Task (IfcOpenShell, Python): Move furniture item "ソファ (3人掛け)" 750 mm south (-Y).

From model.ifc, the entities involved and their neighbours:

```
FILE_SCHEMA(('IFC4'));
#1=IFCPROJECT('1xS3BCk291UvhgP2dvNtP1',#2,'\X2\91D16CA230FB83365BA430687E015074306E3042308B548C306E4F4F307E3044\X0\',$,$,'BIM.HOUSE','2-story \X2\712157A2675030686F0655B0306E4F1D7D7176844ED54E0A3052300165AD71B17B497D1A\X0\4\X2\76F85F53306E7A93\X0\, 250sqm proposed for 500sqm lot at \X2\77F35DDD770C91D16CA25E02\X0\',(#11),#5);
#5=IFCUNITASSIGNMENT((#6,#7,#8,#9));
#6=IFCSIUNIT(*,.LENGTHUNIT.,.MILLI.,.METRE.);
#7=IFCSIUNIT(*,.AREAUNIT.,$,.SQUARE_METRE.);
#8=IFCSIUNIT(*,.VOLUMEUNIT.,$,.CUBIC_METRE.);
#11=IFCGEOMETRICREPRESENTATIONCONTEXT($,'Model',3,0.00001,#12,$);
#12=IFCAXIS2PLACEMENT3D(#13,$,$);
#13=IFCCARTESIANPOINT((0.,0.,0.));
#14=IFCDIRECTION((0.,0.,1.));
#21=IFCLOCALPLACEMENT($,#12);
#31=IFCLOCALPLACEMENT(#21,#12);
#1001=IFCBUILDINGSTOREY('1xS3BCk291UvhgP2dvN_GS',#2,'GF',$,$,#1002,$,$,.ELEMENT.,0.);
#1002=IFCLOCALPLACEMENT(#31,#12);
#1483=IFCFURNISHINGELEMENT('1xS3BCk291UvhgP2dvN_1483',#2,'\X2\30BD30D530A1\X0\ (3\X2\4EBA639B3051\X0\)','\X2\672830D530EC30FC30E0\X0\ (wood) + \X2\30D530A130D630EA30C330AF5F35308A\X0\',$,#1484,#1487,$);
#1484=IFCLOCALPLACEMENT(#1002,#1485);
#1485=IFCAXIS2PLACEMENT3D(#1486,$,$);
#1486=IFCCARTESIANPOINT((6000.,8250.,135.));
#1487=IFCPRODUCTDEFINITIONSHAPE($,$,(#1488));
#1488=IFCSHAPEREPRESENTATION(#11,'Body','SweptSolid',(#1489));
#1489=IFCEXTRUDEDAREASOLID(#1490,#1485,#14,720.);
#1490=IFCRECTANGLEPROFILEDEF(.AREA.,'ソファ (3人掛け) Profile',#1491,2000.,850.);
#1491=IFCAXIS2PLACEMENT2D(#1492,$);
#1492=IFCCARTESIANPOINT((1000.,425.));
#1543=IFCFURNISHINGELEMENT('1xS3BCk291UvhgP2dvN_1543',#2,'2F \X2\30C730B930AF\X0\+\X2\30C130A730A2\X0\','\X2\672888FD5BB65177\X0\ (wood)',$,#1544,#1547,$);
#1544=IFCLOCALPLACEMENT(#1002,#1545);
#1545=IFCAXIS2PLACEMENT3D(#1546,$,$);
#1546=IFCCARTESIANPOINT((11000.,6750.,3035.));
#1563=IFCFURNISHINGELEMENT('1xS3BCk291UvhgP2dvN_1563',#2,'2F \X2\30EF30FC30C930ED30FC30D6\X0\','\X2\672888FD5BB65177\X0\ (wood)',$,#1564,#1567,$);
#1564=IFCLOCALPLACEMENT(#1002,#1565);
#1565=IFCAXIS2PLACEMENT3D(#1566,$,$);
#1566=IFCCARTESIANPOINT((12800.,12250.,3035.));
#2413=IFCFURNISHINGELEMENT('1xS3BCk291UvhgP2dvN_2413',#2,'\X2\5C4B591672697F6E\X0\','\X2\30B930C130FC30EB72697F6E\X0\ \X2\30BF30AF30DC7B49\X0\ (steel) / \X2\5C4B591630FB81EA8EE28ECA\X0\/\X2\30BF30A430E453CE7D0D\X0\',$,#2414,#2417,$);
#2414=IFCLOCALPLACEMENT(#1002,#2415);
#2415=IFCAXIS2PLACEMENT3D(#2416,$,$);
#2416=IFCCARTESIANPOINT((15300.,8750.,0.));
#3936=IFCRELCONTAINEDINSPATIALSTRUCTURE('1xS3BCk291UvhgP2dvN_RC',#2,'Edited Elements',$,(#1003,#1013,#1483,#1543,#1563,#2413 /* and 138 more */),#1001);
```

```python
import ifcopenshell
import ifcopenshell.api.geometry
import ifcopenshell.util.placement
import ifcopenshell.util.unit

model = ifcopenshell.open("model.ifc")
unit_scale = ifcopenshell.util.unit.calculate_unit_scale(model)

item = model.by_guid("1xS3BCk291UvhgP2dvN_1483")
matrix = ifcopenshell.util.placement.get_local_placement(item.ObjectPlacement)
matrix[1, 3] -= 0.75 / unit_scale
ifcopenshell.api.geometry.edit_object_placement(model, product=item, matrix=matrix, is_si=False)

print(ifcopenshell.util.placement.get_local_placement(item.ObjectPlacement).round(3) + 0.0)

model.write("model_v2.ifc")
```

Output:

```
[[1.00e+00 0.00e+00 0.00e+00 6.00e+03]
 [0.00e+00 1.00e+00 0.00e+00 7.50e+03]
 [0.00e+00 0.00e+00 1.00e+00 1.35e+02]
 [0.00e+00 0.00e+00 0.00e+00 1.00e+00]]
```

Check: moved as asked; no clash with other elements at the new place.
